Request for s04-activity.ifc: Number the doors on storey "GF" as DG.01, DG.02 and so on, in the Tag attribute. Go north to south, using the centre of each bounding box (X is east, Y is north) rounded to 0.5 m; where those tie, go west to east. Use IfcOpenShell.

First a look at what the model holds.

```python
import ifcopenshell
import ifcopenshell.util.element
import ifcopenshell.util.placement

model = ifcopenshell.open("s04-activity.ifc")
print(model.schema)
storey = next(s for s in model.by_type("IfcBuildingStorey") if s.Name == "GF")
doors = [e for e in ifcopenshell.util.element.get_decomposition(storey) if e.is_a("IfcDoor")]
for e in sorted(doors, key=lambda e: e.id()):
    origin = ifcopenshell.util.placement.get_local_placement(e.ObjectPlacement)[:3, 3]
    print(e.id(), e.Tag, e.Name, origin.round(2) + 0.0, sep=" | ")
```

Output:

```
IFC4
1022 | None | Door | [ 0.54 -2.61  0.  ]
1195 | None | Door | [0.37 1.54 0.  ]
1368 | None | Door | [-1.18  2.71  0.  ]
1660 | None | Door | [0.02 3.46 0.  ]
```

```python
import ifcopenshell
import ifcopenshell.geom
import ifcopenshell.util.element
import ifcopenshell.util.shape

model = ifcopenshell.open("s04-activity.ifc")
settings = ifcopenshell.geom.settings()
settings.set("use-world-coords", True)


def centre(element):
    shape = ifcopenshell.geom.create_shape(settings, element)
    return ifcopenshell.util.shape.get_bbox_centroid(shape.geometry)


storey = next(s for s in model.by_type("IfcBuildingStorey") if s.Name == "GF")
doors = [e for e in ifcopenshell.util.element.get_decomposition(storey) if e.is_a("IfcDoor")]

# Insertion points can sit at a corner or the storey origin, so sort by the geometry (in metres).
centres = {e: centre(e) for e in doors}
doors.sort(key=lambda e: (-round(centres[e][1] / 0.5), centres[e][0]))

for i, e in enumerate(doors, start=1):
    number = f"DG.{i:02d}"
    e.Tag = number
    print(e.id(), number)

model.write("s04-activity_rev.ifc")
```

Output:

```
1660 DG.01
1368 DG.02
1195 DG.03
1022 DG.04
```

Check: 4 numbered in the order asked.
